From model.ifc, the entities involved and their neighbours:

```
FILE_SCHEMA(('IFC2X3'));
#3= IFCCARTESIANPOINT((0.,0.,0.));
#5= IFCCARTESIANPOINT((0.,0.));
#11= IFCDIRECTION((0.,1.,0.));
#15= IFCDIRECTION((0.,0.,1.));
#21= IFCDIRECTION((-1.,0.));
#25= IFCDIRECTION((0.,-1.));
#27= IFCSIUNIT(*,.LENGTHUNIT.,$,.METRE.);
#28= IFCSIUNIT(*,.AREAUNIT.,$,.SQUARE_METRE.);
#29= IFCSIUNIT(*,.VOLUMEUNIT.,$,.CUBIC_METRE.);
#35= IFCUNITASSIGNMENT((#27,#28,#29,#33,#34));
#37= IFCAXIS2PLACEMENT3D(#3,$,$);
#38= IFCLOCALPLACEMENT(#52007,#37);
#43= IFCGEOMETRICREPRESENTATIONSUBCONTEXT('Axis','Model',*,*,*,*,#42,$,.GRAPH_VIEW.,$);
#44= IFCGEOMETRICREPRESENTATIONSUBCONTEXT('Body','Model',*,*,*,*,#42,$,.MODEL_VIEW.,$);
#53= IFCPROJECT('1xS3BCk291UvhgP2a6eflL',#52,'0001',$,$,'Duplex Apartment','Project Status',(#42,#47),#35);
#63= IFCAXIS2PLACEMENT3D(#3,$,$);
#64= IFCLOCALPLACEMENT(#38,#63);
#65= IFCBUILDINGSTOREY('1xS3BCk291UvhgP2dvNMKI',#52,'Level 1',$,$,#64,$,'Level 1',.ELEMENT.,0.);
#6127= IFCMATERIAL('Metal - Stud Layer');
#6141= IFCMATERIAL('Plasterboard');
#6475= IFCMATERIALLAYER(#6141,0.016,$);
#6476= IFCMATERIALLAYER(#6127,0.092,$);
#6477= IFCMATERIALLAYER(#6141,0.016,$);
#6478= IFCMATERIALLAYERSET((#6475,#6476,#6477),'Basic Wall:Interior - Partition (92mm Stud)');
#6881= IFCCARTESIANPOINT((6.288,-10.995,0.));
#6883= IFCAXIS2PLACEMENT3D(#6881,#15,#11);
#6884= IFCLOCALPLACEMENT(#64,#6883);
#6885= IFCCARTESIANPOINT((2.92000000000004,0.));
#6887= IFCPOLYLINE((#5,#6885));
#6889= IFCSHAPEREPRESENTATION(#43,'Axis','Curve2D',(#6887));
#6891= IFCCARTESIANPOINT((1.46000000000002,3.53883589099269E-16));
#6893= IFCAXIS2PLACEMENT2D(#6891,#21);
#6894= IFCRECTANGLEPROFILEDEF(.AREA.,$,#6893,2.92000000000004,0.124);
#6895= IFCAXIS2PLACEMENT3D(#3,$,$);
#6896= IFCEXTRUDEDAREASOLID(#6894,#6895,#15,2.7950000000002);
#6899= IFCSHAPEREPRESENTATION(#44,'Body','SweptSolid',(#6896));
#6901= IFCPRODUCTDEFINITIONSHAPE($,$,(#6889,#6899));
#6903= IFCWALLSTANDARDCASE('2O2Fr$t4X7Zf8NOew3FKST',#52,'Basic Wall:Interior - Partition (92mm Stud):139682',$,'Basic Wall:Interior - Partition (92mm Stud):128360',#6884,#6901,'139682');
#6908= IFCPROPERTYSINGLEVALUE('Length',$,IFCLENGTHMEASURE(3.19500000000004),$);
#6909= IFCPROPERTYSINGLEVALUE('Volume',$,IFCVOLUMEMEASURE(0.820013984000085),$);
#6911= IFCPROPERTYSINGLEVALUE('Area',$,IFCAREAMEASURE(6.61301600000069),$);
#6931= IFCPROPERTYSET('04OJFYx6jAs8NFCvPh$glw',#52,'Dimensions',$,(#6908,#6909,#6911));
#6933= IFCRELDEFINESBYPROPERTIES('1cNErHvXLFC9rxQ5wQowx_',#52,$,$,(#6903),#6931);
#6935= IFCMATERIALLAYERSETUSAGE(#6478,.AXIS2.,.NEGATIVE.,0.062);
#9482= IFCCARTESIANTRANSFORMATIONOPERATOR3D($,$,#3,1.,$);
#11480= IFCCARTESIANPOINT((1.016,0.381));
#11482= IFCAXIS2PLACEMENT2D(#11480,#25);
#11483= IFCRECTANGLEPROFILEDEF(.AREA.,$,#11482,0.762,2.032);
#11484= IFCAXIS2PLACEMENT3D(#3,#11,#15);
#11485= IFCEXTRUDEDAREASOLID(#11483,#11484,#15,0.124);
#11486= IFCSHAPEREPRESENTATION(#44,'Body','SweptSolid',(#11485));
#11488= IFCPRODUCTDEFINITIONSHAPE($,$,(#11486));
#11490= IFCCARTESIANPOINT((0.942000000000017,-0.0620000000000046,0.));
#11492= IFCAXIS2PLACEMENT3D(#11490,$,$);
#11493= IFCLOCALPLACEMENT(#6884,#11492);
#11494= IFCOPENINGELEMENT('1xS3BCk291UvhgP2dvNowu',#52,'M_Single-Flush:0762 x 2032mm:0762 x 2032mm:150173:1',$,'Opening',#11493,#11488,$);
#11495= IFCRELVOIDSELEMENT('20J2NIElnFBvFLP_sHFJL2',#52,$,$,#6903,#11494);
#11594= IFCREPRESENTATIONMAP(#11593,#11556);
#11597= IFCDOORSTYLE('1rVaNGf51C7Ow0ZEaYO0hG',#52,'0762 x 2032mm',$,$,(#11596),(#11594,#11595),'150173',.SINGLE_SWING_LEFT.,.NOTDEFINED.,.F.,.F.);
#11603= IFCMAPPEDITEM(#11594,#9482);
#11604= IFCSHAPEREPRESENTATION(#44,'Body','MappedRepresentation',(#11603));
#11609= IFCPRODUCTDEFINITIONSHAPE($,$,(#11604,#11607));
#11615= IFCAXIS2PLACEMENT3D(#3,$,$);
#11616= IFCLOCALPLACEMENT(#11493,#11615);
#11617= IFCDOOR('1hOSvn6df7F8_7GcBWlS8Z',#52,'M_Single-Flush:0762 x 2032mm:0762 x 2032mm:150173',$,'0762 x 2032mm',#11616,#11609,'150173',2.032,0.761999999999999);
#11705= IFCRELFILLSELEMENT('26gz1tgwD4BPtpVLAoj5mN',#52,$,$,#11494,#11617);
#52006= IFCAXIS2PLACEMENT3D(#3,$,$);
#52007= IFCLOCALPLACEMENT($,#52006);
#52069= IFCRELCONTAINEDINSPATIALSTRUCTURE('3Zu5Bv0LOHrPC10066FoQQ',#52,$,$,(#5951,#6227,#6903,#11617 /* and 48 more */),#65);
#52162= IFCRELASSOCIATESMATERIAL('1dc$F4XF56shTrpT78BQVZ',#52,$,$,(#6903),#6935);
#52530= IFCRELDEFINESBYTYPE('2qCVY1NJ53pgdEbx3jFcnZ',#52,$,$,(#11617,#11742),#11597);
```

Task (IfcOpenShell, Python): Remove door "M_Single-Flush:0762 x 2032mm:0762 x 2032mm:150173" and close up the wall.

```python
import ifcopenshell
import ifcopenshell.api.feature
import ifcopenshell.api.pset
import ifcopenshell.api.root
import ifcopenshell.geom
import ifcopenshell.util.element
import ifcopenshell.util.shape
import ifcopenshell.util.unit

model = ifcopenshell.open("model.ifc")
area_scale = ifcopenshell.util.unit.calculate_unit_scale(model, "AREAUNIT")
volume_scale = ifcopenshell.util.unit.calculate_unit_scale(model, "VOLUMEUNIT")
settings = ifcopenshell.geom.settings()


def volume(element):
    """Net volume in cubic metres, openings subtracted."""
    shape = ifcopenshell.geom.create_shape(settings, element)
    return ifcopenshell.util.shape.get_volume(shape.geometry)


door = model.by_guid("1hOSvn6df7F8_7GcBWlS8Z")
opening = door.FillsVoids[0].RelatingOpeningElement
wall = opening.VoidsElements[0].RelatingBuildingElement
before = volume(wall)

ifcopenshell.api.root.remove_product(model, product=door)
ifcopenshell.api.feature.remove_feature(model, feature=opening)

after = volume(wall)
thickness = 0.124  # wall thickness in metres

# Update the wall's stored quantities.
pset = model.by_id(ifcopenshell.util.element.get_pset(wall, "Dimensions", should_inherit=False)["id"])
ifcopenshell.api.pset.edit_pset(model, pset=pset, properties={
    "Volume": model.create_entity("IfcVolumeMeasure", after / volume_scale),
    "Area": model.create_entity("IfcAreaMeasure", after / thickness / area_scale),
})

print(f"wall volume {before:.3f} -> {after:.3f} m3")

model.write("model_edited.ifc")
```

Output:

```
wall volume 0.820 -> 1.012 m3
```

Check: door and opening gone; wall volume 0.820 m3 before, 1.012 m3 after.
